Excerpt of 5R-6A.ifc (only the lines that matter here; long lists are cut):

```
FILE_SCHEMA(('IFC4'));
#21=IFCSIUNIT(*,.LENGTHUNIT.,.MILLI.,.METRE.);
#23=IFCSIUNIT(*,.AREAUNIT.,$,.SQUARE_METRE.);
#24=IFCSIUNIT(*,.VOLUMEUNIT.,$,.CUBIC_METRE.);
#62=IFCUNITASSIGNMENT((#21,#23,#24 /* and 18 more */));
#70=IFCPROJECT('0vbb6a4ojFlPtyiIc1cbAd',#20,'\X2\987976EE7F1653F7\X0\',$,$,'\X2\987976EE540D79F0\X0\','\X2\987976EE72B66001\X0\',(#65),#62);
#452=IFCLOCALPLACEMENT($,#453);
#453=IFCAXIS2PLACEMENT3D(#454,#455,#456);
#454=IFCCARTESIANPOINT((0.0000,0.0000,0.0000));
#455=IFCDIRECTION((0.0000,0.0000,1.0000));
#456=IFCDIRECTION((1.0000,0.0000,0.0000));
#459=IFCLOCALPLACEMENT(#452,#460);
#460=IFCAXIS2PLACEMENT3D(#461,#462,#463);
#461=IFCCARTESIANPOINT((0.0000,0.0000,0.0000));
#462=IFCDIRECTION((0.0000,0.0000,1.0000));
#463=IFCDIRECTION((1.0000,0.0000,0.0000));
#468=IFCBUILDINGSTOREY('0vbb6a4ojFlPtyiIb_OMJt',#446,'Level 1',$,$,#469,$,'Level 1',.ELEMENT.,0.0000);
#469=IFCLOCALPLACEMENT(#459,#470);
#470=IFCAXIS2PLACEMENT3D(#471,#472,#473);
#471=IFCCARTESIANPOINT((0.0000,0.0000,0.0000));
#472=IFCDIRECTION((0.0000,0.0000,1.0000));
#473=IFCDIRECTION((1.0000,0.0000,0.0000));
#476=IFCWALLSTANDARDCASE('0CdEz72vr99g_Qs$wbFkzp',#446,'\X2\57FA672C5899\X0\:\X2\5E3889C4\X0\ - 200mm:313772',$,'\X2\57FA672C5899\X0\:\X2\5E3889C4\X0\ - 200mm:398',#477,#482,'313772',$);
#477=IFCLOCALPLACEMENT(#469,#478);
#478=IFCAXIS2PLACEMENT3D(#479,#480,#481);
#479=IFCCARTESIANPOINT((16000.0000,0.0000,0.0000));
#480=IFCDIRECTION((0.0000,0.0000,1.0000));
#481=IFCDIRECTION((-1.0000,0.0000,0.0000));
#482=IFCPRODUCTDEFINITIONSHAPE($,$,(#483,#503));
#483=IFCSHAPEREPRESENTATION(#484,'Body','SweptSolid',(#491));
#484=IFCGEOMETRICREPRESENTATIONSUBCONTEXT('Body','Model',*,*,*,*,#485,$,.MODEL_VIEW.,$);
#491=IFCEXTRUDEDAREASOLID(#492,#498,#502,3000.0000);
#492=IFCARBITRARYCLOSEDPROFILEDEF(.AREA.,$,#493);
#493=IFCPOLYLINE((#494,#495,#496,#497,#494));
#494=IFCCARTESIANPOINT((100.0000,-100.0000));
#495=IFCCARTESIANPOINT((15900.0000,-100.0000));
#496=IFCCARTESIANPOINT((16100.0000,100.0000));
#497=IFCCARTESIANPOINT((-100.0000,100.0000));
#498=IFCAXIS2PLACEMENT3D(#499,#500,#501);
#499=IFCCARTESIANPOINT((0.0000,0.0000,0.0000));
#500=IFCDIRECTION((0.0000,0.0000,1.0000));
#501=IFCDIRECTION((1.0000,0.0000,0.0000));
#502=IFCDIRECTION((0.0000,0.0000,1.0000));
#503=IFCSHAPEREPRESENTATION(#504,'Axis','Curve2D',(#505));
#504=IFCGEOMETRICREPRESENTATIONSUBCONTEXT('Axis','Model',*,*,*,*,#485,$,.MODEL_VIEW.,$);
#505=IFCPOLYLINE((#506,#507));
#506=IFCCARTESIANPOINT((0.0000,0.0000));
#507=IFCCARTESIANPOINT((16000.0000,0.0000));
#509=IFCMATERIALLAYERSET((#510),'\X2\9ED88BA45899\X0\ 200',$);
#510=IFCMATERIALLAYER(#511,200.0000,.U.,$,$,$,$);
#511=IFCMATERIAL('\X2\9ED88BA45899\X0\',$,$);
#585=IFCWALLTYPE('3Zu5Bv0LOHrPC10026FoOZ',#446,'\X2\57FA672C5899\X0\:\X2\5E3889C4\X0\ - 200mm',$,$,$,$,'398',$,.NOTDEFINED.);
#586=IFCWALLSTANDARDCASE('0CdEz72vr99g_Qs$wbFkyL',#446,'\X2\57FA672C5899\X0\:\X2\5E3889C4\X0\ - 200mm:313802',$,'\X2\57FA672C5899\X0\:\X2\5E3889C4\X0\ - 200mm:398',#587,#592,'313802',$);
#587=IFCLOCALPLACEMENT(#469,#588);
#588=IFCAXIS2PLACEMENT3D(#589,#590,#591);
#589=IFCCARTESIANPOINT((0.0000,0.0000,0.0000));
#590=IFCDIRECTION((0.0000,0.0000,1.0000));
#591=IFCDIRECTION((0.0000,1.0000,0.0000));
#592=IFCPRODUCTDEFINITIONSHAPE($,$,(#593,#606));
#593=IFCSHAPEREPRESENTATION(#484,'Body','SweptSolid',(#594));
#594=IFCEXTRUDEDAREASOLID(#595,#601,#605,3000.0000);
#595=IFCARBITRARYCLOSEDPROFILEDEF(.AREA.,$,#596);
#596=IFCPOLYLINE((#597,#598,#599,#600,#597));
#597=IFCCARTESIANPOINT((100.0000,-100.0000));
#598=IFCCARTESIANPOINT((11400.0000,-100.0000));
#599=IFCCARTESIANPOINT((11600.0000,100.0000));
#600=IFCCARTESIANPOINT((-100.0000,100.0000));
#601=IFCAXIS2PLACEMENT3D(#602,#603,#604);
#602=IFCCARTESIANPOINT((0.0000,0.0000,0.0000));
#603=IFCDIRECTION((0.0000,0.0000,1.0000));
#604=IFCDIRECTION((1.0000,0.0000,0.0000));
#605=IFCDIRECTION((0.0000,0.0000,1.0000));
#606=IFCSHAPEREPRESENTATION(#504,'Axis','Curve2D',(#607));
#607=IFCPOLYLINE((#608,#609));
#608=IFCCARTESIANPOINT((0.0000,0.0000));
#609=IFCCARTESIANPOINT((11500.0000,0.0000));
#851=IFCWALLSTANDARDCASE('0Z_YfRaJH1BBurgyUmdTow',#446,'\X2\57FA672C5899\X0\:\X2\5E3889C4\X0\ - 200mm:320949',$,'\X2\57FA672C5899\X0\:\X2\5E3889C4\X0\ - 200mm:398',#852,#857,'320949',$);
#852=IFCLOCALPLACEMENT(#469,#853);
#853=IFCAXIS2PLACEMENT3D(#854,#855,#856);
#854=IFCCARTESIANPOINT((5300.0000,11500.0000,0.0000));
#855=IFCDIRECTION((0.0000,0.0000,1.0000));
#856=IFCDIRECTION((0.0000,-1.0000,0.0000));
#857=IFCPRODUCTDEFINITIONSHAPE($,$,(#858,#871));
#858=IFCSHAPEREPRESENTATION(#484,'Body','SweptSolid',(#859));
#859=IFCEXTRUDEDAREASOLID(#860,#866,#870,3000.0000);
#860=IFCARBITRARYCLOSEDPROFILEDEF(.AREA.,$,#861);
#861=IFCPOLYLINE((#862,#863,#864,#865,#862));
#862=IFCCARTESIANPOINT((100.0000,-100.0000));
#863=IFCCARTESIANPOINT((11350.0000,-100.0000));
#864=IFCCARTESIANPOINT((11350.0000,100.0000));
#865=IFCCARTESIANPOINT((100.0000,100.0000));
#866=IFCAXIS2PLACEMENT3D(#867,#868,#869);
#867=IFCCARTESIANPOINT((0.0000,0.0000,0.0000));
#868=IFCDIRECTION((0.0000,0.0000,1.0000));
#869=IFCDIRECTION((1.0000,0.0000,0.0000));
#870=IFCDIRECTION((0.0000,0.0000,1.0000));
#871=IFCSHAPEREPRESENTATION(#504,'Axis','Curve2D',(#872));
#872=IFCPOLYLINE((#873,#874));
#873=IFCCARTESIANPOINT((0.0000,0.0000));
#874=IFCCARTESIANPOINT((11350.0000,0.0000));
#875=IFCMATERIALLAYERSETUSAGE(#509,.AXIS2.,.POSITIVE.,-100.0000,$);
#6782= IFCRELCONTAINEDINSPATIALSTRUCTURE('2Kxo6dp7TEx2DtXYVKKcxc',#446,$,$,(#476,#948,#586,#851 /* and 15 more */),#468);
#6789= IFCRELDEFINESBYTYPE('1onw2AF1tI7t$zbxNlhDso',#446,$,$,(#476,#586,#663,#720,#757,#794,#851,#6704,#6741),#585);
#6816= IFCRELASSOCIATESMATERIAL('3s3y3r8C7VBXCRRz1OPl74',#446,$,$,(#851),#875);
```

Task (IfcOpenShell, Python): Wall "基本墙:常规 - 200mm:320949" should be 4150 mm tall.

```python
import ifcopenshell
import ifcopenshell.geom
import ifcopenshell.util.representation
import ifcopenshell.util.shape
import ifcopenshell.util.unit

model = ifcopenshell.open("5R-6A.ifc")
unit_scale = ifcopenshell.util.unit.calculate_unit_scale(model)
settings = ifcopenshell.geom.settings()


def volume(element):
    """Net volume in cubic metres, openings subtracted."""
    shape = ifcopenshell.geom.create_shape(settings, element)
    return ifcopenshell.util.shape.get_volume(shape.geometry)


wall = model.by_guid("0Z_YfRaJH1BBurgyUmdTow")
before = volume(wall)

body = ifcopenshell.util.representation.get_representation(wall, "Model", "Body")
solid = body.Items[0]
old_height = solid.Depth
solid.Depth = 4.15 / unit_scale
after = volume(wall)

print(f"height {old_height:g} -> {solid.Depth:g}, volume {before:.3f} -> {after:.3f} m3")

model.write("5R-6A_updated.ifc")
```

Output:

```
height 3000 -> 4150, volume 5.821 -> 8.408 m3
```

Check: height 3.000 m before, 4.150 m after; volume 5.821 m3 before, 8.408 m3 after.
